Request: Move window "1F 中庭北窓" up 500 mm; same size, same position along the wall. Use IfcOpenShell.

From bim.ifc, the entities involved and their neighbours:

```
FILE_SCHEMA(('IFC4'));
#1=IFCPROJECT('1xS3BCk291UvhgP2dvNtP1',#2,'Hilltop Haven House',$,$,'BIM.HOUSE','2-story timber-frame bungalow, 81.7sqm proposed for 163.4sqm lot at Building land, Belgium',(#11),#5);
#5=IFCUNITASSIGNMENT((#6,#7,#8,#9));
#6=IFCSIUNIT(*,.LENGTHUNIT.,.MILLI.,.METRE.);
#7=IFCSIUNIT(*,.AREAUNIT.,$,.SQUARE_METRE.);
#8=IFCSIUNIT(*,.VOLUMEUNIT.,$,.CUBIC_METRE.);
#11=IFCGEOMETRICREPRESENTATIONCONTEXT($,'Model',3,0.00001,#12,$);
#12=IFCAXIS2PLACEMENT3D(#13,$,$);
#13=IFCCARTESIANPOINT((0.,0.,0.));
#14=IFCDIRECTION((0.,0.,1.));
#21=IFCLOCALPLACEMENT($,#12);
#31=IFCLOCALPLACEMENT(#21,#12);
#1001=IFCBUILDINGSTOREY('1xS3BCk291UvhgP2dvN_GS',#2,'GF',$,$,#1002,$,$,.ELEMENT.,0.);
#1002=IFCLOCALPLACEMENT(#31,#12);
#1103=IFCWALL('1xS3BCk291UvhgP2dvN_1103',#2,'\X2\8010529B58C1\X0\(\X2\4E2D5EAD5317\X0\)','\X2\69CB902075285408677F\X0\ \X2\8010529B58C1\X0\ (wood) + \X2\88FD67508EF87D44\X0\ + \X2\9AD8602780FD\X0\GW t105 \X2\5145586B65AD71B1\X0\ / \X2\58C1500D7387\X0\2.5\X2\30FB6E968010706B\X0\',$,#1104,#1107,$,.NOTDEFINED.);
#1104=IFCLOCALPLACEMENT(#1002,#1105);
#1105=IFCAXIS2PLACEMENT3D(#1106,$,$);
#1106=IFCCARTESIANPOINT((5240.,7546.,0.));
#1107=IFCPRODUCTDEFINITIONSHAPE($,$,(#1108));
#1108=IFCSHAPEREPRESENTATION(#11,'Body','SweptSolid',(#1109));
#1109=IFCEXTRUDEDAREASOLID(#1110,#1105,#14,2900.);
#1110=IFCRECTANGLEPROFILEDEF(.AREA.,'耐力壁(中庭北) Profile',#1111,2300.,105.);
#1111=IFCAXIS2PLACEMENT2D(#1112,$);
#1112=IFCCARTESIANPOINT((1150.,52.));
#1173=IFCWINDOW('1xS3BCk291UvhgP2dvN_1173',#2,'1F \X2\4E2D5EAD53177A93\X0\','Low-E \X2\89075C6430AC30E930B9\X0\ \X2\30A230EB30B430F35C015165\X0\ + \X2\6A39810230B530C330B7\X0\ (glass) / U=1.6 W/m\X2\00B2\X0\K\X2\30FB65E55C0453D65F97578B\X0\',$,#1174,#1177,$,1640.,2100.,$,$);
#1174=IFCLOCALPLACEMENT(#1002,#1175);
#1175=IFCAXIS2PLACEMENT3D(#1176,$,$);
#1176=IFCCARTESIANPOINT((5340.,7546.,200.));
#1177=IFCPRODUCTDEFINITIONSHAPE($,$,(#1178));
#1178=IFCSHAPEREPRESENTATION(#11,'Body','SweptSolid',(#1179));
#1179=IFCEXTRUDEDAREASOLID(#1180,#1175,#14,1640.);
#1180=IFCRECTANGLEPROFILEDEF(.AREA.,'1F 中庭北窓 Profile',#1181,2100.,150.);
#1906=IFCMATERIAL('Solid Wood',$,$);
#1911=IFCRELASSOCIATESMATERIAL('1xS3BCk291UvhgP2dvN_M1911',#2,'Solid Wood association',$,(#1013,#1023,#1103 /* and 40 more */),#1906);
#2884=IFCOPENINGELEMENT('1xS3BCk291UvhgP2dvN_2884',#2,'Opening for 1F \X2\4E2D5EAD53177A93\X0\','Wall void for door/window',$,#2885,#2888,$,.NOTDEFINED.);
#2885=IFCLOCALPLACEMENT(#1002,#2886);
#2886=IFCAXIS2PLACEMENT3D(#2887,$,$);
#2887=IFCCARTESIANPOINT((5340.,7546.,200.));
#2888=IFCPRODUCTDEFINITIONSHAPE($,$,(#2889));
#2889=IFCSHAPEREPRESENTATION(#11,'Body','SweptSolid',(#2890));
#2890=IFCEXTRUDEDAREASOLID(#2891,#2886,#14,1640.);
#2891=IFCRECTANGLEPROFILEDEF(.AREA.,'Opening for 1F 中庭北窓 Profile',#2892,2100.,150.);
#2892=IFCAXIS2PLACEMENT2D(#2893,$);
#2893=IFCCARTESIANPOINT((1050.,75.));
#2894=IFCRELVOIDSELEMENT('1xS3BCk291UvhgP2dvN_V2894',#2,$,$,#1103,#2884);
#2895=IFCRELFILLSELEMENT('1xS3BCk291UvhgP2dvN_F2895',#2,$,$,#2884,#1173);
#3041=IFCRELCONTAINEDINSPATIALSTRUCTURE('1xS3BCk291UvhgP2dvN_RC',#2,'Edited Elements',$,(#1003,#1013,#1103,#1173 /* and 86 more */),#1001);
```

```python
import numpy as np
import ifcopenshell
import ifcopenshell.api.geometry
import ifcopenshell.util.placement
import ifcopenshell.util.unit

model = ifcopenshell.open("bim.ifc")
unit_scale = ifcopenshell.util.unit.calculate_unit_scale(model)

window = model.by_guid("1xS3BCk291UvhgP2dvN_1173")
opening = window.FillsVoids[0].RelatingOpeningElement
dz = 0.5 / unit_scale

shift = np.array([0.0, 0.0, dz])
# The window is not placed relative to its opening, so move both.
for product in (opening, window):
    matrix = ifcopenshell.util.placement.get_local_placement(product.ObjectPlacement)
    matrix[:3, 3] += shift
    ifcopenshell.api.geometry.edit_object_placement(model, product=product, matrix=matrix, is_si=False)

print(f"moved by {dz * unit_scale:+.3f} m")

model.write("bim-out.ifc")
```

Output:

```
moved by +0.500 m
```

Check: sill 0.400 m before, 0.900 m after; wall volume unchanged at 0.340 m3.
